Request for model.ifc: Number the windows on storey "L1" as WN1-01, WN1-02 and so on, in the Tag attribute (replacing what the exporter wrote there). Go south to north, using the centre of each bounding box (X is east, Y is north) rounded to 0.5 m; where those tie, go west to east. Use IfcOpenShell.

First a look at what the model holds.

```python
import ifcopenshell
import ifcopenshell.util.element
import ifcopenshell.util.placement

model = ifcopenshell.open("model.ifc")
print(model.schema)
storey = next(s for s in model.by_type("IfcBuildingStorey") if s.Name == "L1")
windows = [e for e in ifcopenshell.util.element.get_decomposition(storey) if e.is_a("IfcWindow")]
for e in sorted(windows, key=lambda e: e.id()):
    origin = ifcopenshell.util.placement.get_local_placement(e.ObjectPlacement)[:3, 3]
    print(e.id(), e.Tag, e.Name, origin.round(2) + 0.0, sep=" | ")
```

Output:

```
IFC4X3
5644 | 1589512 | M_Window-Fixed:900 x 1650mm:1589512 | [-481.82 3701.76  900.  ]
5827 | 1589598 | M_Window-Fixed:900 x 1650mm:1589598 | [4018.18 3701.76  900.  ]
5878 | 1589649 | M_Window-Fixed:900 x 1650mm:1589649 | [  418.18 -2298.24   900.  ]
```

```python
import ifcopenshell
import ifcopenshell.geom
import ifcopenshell.util.element
import ifcopenshell.util.shape

model = ifcopenshell.open("model.ifc")
settings = ifcopenshell.geom.settings()
settings.set("use-world-coords", True)


def centre(element):
    shape = ifcopenshell.geom.create_shape(settings, element)
    return ifcopenshell.util.shape.get_bbox_centroid(shape.geometry)


storey = next(s for s in model.by_type("IfcBuildingStorey") if s.Name == "L1")
windows = [e for e in ifcopenshell.util.element.get_decomposition(storey) if e.is_a("IfcWindow")]

# Insertion points can sit at a corner or the storey origin, so sort by the geometry (in metres).
centres = {e: centre(e) for e in windows}
windows.sort(key=lambda e: (round(centres[e][1] / 0.5), centres[e][0]))

for i, e in enumerate(windows, start=1):
    number = f"WN1-{i:02d}"
    e.Tag = number
    print(e.id(), number)

model.write("model_rev.ifc")
```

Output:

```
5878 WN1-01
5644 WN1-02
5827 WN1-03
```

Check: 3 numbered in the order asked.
